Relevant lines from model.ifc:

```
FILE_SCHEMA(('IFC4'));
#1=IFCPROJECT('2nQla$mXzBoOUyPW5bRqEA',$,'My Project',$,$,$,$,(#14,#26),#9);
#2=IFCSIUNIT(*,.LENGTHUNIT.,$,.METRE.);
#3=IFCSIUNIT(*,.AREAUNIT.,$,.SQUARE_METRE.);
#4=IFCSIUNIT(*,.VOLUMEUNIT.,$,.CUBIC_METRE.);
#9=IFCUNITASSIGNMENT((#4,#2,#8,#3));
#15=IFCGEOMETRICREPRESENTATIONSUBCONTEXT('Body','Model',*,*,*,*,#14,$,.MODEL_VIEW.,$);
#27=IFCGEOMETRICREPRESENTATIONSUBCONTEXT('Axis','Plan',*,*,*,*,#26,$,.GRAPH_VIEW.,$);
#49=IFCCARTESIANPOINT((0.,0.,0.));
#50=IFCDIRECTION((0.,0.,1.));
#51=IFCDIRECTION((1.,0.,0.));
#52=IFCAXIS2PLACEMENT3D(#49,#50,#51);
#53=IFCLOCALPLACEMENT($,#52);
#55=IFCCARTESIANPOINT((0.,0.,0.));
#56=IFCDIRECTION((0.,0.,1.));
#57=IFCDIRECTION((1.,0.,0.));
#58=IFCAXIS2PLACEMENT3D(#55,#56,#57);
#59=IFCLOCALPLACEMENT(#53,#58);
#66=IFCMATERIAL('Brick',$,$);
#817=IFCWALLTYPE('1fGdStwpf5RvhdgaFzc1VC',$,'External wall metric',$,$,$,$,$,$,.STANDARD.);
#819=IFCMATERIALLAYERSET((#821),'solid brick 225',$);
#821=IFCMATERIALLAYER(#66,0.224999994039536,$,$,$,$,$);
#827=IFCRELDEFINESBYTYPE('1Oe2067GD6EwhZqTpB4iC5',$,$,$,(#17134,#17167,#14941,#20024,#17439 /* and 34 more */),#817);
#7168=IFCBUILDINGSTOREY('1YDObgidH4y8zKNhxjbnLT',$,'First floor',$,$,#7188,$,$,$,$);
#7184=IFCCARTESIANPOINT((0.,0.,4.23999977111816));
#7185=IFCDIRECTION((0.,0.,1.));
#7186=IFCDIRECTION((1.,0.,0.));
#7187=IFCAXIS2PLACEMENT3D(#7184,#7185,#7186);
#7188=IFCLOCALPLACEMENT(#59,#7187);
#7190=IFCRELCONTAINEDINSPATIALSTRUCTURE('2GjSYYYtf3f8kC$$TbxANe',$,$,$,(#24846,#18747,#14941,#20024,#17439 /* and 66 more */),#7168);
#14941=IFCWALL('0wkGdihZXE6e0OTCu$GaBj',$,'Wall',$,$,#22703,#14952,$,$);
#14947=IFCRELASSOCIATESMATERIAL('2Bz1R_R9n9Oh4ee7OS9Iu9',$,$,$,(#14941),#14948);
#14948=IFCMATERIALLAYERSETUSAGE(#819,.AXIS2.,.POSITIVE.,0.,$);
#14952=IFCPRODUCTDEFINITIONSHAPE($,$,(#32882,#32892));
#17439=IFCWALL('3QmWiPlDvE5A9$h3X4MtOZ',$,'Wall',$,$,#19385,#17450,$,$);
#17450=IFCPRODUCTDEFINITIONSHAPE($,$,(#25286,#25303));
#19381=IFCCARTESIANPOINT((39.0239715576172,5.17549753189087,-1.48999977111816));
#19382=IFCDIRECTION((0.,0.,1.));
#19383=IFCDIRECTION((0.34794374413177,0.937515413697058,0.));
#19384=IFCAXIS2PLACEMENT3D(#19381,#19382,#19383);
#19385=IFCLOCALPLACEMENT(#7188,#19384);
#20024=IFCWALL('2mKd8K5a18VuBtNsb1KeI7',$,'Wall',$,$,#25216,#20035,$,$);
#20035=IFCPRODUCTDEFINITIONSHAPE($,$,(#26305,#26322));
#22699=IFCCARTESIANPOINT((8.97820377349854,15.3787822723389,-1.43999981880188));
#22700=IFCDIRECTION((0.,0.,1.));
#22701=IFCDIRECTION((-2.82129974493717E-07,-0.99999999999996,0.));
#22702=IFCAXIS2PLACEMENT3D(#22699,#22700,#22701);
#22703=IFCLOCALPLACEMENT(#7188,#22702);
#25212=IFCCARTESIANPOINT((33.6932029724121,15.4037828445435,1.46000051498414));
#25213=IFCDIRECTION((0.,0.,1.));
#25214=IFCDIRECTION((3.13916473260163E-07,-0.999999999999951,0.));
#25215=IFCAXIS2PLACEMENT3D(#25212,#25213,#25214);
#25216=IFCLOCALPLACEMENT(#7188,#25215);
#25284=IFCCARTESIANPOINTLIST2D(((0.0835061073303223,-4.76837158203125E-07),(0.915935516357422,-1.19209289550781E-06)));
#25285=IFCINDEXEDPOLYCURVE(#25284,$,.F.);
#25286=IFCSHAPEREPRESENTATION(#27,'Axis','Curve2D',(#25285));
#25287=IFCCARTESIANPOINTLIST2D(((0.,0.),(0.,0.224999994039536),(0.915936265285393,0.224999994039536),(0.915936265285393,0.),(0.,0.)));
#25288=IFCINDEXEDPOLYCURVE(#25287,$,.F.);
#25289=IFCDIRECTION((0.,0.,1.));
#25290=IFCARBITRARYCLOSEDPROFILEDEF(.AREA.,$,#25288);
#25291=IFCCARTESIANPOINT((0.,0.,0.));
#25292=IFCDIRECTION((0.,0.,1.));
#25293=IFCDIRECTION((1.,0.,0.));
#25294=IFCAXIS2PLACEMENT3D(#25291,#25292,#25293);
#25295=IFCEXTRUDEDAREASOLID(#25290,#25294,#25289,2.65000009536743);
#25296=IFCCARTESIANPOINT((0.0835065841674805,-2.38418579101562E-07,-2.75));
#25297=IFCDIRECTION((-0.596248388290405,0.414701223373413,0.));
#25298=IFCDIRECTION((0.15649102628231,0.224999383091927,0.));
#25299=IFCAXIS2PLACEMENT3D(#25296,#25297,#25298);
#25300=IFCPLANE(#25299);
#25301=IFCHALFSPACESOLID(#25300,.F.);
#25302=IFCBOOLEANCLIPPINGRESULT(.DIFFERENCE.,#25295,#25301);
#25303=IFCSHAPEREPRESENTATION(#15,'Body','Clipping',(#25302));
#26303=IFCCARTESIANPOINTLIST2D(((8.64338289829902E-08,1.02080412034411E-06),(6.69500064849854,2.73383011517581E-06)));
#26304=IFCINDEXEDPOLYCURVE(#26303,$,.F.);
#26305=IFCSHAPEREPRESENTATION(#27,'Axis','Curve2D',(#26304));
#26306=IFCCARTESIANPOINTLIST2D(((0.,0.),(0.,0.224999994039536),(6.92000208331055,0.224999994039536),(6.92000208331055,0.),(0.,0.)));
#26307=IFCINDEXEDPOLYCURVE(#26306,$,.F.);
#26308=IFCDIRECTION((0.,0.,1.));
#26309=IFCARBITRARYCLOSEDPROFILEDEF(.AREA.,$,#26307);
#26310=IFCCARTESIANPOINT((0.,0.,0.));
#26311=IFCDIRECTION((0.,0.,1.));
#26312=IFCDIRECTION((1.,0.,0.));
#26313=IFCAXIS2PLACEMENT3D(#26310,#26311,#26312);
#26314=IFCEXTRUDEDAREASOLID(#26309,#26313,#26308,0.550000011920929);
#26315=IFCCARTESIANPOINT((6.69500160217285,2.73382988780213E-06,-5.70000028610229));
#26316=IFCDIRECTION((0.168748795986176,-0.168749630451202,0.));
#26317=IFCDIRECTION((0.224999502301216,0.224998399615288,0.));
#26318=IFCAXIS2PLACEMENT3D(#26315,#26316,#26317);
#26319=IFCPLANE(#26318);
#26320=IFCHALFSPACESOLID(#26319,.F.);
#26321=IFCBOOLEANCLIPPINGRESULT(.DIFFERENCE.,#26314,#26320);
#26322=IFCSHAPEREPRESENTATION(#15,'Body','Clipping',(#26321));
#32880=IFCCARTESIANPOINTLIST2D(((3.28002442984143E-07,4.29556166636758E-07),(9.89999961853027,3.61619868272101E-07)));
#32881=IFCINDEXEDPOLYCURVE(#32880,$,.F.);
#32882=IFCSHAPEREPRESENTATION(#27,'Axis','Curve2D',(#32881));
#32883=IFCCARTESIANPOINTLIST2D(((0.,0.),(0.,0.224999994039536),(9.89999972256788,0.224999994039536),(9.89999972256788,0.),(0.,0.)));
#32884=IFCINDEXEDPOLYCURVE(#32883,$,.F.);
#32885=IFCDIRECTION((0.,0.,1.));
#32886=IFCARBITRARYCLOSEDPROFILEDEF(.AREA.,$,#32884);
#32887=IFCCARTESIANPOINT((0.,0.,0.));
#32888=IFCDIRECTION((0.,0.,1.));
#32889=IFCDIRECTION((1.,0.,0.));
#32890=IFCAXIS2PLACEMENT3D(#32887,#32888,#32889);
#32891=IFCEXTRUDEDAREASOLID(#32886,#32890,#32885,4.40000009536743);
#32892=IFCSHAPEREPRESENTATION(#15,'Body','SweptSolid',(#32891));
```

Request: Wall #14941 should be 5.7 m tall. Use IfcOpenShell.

```python
import ifcopenshell
import ifcopenshell.geom
import ifcopenshell.util.representation
import ifcopenshell.util.shape

model = ifcopenshell.open("model.ifc")
settings = ifcopenshell.geom.settings()


def volume(element):
    """Net volume in cubic metres, openings subtracted."""
    shape = ifcopenshell.geom.create_shape(settings, element)
    return ifcopenshell.util.shape.get_volume(shape.geometry)


wall = model.by_guid("0wkGdihZXE6e0OTCu$GaBj")
before = volume(wall)

body = ifcopenshell.util.representation.get_representation(wall, "Model", "Body")
solid = body.Items[0]
old_height = solid.Depth
solid.Depth = 5.7
after = volume(wall)

print(f"height {old_height:g} -> {solid.Depth:g}, volume {before:.3f} -> {after:.3f} m3")

model.write("model_edited.ifc")
```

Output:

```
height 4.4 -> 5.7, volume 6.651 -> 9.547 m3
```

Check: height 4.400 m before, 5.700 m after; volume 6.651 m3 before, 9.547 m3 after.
